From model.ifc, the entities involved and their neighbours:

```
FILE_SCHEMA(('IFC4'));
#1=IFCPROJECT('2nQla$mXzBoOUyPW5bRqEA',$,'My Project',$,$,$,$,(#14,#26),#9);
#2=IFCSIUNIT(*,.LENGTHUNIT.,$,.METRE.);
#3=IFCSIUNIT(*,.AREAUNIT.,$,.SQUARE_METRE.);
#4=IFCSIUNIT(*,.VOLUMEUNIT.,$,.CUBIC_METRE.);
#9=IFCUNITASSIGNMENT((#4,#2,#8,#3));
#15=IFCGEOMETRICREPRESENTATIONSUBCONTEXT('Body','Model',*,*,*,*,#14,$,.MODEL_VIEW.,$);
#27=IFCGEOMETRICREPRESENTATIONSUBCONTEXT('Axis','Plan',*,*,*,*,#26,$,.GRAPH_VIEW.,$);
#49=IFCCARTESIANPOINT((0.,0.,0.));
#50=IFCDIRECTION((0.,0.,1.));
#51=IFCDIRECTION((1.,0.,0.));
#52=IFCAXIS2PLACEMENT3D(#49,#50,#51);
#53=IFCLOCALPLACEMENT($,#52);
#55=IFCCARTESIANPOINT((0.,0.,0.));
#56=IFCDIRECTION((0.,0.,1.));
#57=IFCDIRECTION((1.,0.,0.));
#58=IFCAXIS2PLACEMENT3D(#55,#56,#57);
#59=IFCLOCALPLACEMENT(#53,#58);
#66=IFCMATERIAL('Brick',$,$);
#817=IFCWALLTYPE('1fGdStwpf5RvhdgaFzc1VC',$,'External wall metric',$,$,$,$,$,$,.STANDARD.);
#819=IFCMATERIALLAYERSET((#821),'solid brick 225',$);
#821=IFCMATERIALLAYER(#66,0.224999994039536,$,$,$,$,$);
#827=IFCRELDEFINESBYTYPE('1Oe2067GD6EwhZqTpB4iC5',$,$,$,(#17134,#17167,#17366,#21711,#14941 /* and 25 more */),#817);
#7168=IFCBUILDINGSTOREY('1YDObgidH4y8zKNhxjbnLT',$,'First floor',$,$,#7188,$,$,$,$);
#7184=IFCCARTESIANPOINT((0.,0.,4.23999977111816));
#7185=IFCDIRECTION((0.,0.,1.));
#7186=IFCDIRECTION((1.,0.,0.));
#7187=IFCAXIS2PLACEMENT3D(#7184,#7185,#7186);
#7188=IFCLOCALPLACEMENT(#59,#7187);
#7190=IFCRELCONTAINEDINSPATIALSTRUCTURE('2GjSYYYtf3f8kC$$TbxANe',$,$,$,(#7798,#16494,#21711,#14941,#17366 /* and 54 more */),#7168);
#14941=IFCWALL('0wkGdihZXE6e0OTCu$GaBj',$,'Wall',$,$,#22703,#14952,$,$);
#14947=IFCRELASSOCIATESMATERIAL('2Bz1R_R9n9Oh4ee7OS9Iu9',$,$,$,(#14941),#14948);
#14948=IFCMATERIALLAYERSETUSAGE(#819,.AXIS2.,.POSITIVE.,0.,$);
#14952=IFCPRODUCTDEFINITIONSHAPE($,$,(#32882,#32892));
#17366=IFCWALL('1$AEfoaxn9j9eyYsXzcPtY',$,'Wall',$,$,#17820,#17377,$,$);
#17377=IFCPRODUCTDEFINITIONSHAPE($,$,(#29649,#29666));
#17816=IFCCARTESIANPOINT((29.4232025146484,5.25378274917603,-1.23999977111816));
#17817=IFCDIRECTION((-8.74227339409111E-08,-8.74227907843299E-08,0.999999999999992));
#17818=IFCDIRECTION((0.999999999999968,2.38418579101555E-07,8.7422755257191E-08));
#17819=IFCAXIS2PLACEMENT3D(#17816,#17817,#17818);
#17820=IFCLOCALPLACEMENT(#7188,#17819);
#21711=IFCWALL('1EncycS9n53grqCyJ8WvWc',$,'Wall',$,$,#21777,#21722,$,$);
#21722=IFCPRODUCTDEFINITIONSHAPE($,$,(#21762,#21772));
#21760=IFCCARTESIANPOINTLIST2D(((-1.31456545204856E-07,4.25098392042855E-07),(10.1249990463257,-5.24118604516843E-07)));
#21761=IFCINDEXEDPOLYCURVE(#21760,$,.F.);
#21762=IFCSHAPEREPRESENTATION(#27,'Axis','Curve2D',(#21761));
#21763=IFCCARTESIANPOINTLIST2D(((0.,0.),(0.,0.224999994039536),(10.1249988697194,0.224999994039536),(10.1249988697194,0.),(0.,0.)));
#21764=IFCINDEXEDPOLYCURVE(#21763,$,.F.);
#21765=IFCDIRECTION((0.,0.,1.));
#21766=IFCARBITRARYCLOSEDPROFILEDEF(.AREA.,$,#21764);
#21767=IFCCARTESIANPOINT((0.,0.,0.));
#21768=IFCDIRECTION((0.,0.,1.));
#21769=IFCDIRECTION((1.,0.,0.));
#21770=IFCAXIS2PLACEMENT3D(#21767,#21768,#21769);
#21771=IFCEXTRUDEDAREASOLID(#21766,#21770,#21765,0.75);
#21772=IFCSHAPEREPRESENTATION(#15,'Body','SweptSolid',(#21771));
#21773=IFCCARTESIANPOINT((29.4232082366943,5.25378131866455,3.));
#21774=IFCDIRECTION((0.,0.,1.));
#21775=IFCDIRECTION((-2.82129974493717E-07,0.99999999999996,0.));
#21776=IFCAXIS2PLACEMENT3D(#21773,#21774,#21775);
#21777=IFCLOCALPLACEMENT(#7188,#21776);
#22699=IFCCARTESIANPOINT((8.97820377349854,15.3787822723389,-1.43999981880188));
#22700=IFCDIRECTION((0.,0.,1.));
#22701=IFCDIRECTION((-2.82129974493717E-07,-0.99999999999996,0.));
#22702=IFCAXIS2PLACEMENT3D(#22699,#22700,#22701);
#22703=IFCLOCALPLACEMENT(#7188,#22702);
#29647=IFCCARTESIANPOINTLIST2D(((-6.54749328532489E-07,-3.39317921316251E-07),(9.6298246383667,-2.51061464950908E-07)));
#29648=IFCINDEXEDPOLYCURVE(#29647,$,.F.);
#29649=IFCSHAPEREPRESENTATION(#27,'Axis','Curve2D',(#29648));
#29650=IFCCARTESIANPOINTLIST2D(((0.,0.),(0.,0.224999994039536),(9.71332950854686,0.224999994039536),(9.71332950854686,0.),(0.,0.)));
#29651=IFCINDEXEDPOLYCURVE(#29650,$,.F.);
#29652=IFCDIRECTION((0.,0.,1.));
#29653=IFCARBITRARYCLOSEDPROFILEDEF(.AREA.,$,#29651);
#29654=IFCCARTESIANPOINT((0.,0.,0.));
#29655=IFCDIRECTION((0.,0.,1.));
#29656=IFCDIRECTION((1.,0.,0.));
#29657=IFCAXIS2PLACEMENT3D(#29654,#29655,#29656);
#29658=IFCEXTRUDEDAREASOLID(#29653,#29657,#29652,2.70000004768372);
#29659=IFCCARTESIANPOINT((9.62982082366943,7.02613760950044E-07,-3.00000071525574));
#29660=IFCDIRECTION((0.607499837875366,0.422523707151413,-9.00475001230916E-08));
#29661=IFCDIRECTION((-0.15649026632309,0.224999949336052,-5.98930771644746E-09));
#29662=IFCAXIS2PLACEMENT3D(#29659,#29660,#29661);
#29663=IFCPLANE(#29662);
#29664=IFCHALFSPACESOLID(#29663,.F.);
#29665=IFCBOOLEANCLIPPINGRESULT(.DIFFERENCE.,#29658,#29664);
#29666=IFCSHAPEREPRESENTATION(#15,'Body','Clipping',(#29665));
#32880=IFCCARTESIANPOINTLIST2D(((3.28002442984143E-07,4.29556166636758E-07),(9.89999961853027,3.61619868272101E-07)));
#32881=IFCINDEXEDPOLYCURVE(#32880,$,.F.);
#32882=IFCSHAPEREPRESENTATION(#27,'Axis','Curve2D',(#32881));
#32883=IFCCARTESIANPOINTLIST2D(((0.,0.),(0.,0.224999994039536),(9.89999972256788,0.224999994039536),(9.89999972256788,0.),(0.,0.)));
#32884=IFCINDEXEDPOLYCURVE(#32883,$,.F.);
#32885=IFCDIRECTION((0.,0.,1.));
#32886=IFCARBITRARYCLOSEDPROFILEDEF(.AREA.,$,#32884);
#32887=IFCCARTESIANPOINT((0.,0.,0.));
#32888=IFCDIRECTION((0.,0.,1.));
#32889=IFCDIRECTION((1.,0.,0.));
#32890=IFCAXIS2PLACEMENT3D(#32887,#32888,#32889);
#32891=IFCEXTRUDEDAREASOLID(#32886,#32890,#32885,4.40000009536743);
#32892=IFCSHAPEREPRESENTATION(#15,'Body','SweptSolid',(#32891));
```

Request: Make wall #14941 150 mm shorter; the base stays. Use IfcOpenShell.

```python
import ifcopenshell
import ifcopenshell.geom
import ifcopenshell.util.representation
import ifcopenshell.util.shape
import ifcopenshell.util.unit

model = ifcopenshell.open("model.ifc")
unit_scale = ifcopenshell.util.unit.calculate_unit_scale(model)
settings = ifcopenshell.geom.settings()


def volume(element):
    """Net volume in cubic metres, openings subtracted."""
    shape = ifcopenshell.geom.create_shape(settings, element)
    return ifcopenshell.util.shape.get_volume(shape.geometry)


wall = model.by_id(14941)
before = volume(wall)

body = ifcopenshell.util.representation.get_representation(wall, "Model", "Body")
solid = body.Items[0]
old_height = solid.Depth
solid.Depth -= 0.15 / unit_scale
after = volume(wall)

print(f"height {old_height:g} -> {solid.Depth:g}, volume {before:.3f} -> {after:.3f} m3")

model.write("model_edited.ifc")
```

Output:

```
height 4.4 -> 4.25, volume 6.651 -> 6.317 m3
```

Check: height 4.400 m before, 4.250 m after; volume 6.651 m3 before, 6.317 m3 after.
